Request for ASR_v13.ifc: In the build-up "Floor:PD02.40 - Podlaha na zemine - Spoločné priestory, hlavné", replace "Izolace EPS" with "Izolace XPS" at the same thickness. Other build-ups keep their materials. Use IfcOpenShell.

First a look at what the model holds.

```python
import ifcopenshell
import ifcopenshell.util.element

model = ifcopenshell.open("ASR_v13.ifc")
print(model.schema)
for layer_set in model.by_type("IfcMaterialLayerSet"):
    if layer_set.LayerSetName == "Floor:PD02.40 - Podlaha na zemine - Spoločné priestory, hlavné":
        for layer in layer_set.MaterialLayers:
            print(layer.id(), layer.Material and layer.Material.Name, layer.LayerThickness, sep=" | ")
        print(len(ifcopenshell.util.element.get_elements_by_material(model, layer_set)), "elements and types use it")
print(sorted(m.Name for m in model.by_type("IfcMaterial") if m.Name)[:60])
```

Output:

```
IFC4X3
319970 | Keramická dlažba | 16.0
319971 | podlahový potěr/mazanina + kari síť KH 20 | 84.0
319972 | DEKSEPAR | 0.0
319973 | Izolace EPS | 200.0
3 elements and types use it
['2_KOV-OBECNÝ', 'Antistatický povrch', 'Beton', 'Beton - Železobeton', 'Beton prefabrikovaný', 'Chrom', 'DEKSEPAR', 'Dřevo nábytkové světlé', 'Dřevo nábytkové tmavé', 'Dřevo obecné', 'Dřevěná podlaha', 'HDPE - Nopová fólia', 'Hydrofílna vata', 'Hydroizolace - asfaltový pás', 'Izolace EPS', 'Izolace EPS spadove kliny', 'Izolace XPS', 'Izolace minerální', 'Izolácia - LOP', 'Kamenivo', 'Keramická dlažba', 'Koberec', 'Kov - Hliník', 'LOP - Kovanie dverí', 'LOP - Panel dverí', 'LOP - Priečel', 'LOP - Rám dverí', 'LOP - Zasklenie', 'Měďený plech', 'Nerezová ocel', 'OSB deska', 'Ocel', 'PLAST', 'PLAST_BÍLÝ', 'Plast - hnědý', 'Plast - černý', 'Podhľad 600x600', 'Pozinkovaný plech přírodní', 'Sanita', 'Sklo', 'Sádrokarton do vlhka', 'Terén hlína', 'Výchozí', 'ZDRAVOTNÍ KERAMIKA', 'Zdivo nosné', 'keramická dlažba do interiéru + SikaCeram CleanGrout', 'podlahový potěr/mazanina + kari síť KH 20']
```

```python
import ifcopenshell
import ifcopenshell.api.material

model = ifcopenshell.open("ASR_v13.ifc")

layer_set = next(s for s in model.by_type("IfcMaterialLayerSet") if s.LayerSetName == "Floor:PD02.40 - Podlaha na zemine - Spoločné priestory, hlavné")
layer = next(l for l in layer_set.MaterialLayers if l.Material and l.Material.Name == "Izolace EPS")
material = next(m for m in model.by_type("IfcMaterial") if m.Name == "Izolace XPS")

# Point this one layer at the other material; renaming the old one would change it everywhere.
ifcopenshell.api.material.edit_layer(model, layer=layer, attributes={"Name": material.Name}, material=material)

print([l.Material.Name if l.Material else None for l in layer_set.MaterialLayers])

model.write("ASR_v13_edited.ifc")
```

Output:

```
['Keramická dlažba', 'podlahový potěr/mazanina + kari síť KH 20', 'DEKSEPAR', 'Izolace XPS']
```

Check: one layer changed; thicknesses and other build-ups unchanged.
